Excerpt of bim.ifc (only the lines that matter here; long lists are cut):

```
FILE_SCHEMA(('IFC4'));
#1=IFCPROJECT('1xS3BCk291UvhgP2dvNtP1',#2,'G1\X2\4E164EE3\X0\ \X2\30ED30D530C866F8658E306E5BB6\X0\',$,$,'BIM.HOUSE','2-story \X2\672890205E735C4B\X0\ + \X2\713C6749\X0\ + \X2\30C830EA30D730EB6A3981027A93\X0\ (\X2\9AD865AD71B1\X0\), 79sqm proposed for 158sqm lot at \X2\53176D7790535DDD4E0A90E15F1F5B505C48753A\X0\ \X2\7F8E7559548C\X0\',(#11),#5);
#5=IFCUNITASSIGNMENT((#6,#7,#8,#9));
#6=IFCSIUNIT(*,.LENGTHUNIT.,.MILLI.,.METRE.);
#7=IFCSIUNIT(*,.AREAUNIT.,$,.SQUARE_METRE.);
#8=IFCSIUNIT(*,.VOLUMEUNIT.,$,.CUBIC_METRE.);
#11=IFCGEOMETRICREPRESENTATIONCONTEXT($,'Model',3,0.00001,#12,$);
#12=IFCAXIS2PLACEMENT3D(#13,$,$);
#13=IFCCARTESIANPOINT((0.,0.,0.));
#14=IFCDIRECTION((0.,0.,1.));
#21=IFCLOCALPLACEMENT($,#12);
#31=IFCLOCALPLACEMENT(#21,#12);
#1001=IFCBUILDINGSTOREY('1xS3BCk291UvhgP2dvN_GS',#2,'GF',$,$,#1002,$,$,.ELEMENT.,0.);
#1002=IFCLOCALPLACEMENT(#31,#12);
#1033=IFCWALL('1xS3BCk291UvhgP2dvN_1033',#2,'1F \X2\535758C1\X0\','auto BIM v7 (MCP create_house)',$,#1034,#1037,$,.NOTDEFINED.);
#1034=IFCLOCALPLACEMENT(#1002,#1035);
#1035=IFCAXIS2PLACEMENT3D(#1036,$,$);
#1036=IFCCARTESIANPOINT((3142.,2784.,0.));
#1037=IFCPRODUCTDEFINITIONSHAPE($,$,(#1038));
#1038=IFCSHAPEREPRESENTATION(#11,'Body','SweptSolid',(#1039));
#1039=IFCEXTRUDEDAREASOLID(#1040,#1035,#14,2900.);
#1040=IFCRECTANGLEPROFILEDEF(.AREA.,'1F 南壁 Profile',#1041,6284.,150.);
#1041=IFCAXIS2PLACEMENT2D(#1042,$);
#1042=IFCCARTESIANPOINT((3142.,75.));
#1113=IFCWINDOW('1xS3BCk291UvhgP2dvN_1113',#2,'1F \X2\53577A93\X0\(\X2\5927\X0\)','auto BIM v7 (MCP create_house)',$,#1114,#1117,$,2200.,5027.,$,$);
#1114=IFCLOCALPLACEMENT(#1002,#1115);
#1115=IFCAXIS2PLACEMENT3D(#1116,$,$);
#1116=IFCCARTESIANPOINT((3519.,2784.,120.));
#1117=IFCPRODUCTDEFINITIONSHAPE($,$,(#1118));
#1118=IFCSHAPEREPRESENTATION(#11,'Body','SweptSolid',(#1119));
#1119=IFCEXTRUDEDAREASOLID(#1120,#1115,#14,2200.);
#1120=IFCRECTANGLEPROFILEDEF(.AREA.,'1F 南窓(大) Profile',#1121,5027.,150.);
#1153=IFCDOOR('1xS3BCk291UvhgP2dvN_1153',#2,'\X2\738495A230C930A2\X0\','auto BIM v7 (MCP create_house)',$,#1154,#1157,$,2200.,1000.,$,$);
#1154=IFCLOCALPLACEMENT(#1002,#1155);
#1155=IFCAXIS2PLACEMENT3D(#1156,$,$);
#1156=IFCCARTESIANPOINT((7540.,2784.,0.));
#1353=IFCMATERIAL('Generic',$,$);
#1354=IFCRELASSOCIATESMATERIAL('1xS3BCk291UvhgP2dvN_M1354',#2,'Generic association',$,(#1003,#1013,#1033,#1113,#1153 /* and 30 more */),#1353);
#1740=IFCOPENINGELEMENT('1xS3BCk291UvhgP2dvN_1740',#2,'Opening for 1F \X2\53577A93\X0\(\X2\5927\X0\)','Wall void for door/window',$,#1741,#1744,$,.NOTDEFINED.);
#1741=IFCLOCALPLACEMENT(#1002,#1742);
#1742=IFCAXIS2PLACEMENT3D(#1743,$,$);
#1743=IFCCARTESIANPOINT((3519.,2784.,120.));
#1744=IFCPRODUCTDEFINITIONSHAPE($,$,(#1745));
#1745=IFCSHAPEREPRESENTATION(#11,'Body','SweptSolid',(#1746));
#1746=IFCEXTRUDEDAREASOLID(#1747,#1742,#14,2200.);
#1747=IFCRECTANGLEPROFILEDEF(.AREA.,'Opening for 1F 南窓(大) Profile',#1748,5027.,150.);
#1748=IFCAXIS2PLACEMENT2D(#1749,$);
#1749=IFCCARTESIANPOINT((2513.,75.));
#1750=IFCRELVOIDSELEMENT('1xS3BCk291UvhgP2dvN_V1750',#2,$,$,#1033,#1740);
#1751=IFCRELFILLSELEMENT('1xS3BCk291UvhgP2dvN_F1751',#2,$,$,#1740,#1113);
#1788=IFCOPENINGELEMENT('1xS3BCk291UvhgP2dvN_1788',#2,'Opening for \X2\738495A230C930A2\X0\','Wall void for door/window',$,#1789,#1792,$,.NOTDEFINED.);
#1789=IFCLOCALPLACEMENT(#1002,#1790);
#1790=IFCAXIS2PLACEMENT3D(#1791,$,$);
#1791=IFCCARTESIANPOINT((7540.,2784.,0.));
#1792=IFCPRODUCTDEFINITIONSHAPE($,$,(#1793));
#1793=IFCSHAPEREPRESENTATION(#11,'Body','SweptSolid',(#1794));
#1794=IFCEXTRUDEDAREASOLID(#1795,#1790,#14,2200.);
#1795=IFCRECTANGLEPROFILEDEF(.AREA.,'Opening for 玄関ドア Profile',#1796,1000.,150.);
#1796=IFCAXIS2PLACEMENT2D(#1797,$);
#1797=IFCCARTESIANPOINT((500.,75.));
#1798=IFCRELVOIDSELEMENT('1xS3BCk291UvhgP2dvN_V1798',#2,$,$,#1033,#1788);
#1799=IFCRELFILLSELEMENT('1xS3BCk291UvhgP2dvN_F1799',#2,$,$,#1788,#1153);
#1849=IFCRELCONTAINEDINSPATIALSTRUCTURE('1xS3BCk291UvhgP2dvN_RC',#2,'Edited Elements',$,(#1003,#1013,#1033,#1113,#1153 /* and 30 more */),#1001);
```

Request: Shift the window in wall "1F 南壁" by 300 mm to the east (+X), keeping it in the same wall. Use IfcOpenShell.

```python
import ifcopenshell
import ifcopenshell.api.geometry
import ifcopenshell.util.placement
import ifcopenshell.util.unit

model = ifcopenshell.open("bim.ifc")
unit_scale = ifcopenshell.util.unit.calculate_unit_scale(model)

window = model.by_guid("1xS3BCk291UvhgP2dvN_1113")
opening = window.FillsVoids[0].RelatingOpeningElement
wall = opening.VoidsElements[0].RelatingBuildingElement

wall_matrix = ifcopenshell.util.placement.get_local_placement(wall.ObjectPlacement)
shift = wall_matrix[:3, 0] * 0.3 / unit_scale
before = ifcopenshell.util.placement.get_local_placement(window.ObjectPlacement)[:3, 3].copy()

# The window is not placed relative to its opening, so move both.
for product in (opening, window):
    matrix = ifcopenshell.util.placement.get_local_placement(product.ObjectPlacement)
    matrix[:3, 3] += shift
    ifcopenshell.api.geometry.edit_object_placement(model, product=product, matrix=matrix, is_si=False)

after = ifcopenshell.util.placement.get_local_placement(window.ObjectPlacement)[:3, 3]
print("window moved by", (after - before).round(3) + 0.0)

model.write("bim_rev.ifc")
```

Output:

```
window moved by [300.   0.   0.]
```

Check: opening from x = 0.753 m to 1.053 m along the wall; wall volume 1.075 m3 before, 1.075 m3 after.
